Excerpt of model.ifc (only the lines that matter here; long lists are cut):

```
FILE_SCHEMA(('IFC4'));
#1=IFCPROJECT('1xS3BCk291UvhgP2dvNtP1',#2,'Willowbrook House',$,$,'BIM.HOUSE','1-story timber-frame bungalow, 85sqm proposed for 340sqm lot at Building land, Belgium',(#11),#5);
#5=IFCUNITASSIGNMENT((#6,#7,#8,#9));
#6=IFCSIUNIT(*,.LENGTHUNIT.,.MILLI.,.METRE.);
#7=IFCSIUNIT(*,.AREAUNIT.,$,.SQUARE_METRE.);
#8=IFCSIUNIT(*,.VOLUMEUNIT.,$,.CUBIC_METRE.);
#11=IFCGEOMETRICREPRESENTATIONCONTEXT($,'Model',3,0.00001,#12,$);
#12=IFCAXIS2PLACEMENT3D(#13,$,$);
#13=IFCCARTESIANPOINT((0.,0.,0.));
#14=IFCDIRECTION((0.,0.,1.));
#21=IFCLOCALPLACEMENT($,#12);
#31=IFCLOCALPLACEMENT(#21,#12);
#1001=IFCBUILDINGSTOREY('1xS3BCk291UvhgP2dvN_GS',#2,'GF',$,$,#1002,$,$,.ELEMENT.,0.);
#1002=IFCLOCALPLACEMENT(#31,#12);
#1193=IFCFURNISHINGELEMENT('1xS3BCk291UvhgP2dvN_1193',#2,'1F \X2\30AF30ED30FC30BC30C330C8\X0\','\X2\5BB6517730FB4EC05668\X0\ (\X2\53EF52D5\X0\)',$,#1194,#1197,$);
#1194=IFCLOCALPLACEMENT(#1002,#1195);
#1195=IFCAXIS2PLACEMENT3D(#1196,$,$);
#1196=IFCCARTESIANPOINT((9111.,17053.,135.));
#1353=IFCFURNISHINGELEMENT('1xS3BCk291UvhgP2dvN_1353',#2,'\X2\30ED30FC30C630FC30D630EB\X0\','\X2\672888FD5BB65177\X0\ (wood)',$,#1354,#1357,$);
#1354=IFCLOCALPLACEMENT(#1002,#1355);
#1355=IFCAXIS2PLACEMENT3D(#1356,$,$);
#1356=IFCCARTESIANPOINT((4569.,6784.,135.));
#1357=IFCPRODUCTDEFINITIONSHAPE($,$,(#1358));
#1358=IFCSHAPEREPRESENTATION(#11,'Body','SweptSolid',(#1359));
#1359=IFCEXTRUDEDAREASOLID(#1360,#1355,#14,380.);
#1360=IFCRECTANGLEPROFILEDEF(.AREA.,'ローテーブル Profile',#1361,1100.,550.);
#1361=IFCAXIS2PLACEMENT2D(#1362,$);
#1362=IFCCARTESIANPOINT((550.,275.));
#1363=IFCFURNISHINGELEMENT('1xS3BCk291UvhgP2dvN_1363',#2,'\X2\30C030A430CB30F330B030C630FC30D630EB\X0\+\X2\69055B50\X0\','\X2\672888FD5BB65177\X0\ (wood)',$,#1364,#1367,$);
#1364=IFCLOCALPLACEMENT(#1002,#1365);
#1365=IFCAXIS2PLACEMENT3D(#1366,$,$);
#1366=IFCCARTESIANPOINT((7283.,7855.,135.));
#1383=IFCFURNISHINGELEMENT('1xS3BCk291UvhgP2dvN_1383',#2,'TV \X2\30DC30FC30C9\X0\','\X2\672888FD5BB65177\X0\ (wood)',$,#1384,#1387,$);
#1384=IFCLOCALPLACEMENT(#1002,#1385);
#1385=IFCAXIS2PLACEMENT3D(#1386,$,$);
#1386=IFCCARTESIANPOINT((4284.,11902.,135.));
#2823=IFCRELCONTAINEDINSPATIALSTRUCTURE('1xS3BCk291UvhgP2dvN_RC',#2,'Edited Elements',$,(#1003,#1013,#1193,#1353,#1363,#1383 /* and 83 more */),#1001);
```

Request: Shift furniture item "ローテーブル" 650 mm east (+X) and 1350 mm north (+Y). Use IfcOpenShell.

```python
import ifcopenshell
import ifcopenshell.api.geometry
import ifcopenshell.util.placement
import ifcopenshell.util.unit

model = ifcopenshell.open("model.ifc")
unit_scale = ifcopenshell.util.unit.calculate_unit_scale(model)

item = model.by_id(1353)
matrix = ifcopenshell.util.placement.get_local_placement(item.ObjectPlacement)
matrix[0, 3] += 0.65 / unit_scale
matrix[1, 3] += 1.35 / unit_scale
ifcopenshell.api.geometry.edit_object_placement(model, product=item, matrix=matrix, is_si=False)

print(ifcopenshell.util.placement.get_local_placement(item.ObjectPlacement).round(3) + 0.0)

model.write("model-out.ifc")
```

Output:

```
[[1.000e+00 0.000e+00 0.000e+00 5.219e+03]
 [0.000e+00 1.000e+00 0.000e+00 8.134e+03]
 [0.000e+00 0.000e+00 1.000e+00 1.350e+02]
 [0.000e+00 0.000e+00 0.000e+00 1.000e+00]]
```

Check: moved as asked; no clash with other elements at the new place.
